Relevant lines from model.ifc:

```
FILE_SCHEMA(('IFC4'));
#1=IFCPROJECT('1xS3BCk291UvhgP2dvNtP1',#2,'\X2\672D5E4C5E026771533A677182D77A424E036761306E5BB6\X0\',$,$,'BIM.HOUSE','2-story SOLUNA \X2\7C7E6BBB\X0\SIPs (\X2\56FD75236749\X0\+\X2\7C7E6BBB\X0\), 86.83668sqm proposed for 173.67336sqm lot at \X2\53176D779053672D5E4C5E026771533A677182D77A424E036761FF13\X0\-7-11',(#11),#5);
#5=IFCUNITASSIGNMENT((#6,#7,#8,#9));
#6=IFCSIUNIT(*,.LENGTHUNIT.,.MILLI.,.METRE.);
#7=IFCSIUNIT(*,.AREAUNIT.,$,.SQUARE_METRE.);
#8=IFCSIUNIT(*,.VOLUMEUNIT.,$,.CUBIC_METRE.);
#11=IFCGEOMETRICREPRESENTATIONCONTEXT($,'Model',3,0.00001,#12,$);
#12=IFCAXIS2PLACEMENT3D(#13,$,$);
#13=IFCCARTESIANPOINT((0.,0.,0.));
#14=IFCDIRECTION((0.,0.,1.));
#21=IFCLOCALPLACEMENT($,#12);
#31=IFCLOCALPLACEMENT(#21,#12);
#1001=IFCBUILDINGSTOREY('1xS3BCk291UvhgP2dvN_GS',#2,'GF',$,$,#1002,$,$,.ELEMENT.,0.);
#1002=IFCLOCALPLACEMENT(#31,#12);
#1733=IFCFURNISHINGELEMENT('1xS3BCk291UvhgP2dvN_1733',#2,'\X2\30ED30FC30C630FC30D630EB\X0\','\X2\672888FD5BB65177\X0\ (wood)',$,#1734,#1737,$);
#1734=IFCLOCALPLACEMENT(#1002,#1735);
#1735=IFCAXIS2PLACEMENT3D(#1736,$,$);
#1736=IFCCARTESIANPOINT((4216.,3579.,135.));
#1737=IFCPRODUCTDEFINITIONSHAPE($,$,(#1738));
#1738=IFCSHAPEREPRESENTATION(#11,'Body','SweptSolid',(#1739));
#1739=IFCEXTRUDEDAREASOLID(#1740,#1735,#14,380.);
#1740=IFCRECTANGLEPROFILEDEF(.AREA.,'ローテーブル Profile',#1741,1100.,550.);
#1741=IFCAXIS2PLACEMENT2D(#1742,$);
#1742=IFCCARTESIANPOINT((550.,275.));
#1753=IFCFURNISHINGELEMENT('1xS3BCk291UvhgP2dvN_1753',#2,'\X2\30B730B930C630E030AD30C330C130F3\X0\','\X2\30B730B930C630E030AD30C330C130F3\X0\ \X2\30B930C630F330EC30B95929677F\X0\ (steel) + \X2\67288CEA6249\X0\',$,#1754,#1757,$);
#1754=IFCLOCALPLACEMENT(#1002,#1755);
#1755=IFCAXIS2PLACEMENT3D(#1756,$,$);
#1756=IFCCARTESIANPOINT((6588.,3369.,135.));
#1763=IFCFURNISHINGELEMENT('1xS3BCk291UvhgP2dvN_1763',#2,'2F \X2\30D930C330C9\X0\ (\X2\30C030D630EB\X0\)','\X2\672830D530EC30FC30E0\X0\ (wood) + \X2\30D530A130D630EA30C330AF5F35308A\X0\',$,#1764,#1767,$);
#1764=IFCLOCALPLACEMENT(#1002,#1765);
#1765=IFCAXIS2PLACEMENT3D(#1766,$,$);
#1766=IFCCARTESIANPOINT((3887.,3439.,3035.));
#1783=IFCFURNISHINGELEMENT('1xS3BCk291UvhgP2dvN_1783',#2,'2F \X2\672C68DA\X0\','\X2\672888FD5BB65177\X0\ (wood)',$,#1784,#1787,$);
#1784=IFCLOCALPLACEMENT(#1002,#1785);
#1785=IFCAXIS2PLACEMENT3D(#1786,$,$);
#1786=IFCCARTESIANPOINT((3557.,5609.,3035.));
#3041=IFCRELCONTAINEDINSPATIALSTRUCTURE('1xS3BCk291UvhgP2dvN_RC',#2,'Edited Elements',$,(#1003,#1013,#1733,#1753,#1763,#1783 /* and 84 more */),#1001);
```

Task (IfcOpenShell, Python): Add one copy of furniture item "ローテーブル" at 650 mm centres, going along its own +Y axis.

```python
import ifcopenshell
import ifcopenshell.api.geometry
import ifcopenshell.api.root
import ifcopenshell.util.element
import ifcopenshell.util.placement
import ifcopenshell.util.unit

model = ifcopenshell.open("model.ifc")
unit_scale = ifcopenshell.util.unit.calculate_unit_scale(model)


def reuse_history(source, copy):
    """copy_class also copies each property set's owner history, people and application; keep the originals."""
    for rel in copy.IsDefinedBy:
        if rel.is_a("IfcRelDefinesByProperties") and (history := rel.RelatingPropertyDefinition.OwnerHistory):
            rel.RelatingPropertyDefinition.OwnerHistory = source.OwnerHistory
            ifcopenshell.util.element.remove_deep2(model, history)


source = model.by_id(1733)
base = ifcopenshell.util.placement.get_local_placement(source.ObjectPlacement)
step = base[:3, 1] * 0.65 / unit_scale

for i in range(1, 2):
    copy = ifcopenshell.api.root.copy_class(model, product=source)
    copy.Representation = ifcopenshell.util.element.copy_deep(
        model, source.Representation, exclude=["IfcGeometricRepresentationContext", "IfcRepresentationMap"]
    )
    reuse_history(source, copy)
    matrix = base.copy()
    matrix[:3, 3] += i * step
    print("added at", matrix[:3, 3].round(3) + 0.0)
    ifcopenshell.api.geometry.edit_object_placement(model, product=copy, matrix=matrix, is_si=False)

model.write("model-out.ifc")
```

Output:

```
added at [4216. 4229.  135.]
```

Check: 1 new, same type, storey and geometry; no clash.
